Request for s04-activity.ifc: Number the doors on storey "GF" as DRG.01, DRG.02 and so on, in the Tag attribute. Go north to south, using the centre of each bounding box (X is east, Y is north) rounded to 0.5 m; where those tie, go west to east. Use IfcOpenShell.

First a look at what the model holds.

```python
import ifcopenshell
import ifcopenshell.util.element
import ifcopenshell.util.placement

model = ifcopenshell.open("s04-activity.ifc")
print(model.schema)
storey = next(s for s in model.by_type("IfcBuildingStorey") if s.Name == "GF")
doors = [e for e in ifcopenshell.util.element.get_decomposition(storey) if e.is_a("IfcDoor")]
for e in sorted(doors, key=lambda e: e.id()):
    origin = ifcopenshell.util.placement.get_local_placement(e.ObjectPlacement)[:3, 3]
    print(e.id(), e.Tag, e.Name, origin.round(2) + 0.0, sep=" | ")
```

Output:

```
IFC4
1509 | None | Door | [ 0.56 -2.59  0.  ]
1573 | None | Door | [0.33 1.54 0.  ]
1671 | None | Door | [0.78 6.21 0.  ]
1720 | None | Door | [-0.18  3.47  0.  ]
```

```python
import ifcopenshell
import ifcopenshell.geom
import ifcopenshell.util.element
import ifcopenshell.util.shape

model = ifcopenshell.open("s04-activity.ifc")
settings = ifcopenshell.geom.settings()
settings.set("use-world-coords", True)


def centre(element):
    shape = ifcopenshell.geom.create_shape(settings, element)
    return ifcopenshell.util.shape.get_bbox_centroid(shape.geometry)


storey = next(s for s in model.by_type("IfcBuildingStorey") if s.Name == "GF")
doors = [e for e in ifcopenshell.util.element.get_decomposition(storey) if e.is_a("IfcDoor")]

# Insertion points can sit at a corner or the storey origin, so sort by the geometry (in metres).
centres = {e: centre(e) for e in doors}
doors.sort(key=lambda e: (-round(centres[e][1] / 0.5), centres[e][0]))

for i, e in enumerate(doors, start=1):
    number = f"DRG.{i:02d}"
    e.Tag = number
    print(e.id(), number)

model.write("s04-activity_edited.ifc")
```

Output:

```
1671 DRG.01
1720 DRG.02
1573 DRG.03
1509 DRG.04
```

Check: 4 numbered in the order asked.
